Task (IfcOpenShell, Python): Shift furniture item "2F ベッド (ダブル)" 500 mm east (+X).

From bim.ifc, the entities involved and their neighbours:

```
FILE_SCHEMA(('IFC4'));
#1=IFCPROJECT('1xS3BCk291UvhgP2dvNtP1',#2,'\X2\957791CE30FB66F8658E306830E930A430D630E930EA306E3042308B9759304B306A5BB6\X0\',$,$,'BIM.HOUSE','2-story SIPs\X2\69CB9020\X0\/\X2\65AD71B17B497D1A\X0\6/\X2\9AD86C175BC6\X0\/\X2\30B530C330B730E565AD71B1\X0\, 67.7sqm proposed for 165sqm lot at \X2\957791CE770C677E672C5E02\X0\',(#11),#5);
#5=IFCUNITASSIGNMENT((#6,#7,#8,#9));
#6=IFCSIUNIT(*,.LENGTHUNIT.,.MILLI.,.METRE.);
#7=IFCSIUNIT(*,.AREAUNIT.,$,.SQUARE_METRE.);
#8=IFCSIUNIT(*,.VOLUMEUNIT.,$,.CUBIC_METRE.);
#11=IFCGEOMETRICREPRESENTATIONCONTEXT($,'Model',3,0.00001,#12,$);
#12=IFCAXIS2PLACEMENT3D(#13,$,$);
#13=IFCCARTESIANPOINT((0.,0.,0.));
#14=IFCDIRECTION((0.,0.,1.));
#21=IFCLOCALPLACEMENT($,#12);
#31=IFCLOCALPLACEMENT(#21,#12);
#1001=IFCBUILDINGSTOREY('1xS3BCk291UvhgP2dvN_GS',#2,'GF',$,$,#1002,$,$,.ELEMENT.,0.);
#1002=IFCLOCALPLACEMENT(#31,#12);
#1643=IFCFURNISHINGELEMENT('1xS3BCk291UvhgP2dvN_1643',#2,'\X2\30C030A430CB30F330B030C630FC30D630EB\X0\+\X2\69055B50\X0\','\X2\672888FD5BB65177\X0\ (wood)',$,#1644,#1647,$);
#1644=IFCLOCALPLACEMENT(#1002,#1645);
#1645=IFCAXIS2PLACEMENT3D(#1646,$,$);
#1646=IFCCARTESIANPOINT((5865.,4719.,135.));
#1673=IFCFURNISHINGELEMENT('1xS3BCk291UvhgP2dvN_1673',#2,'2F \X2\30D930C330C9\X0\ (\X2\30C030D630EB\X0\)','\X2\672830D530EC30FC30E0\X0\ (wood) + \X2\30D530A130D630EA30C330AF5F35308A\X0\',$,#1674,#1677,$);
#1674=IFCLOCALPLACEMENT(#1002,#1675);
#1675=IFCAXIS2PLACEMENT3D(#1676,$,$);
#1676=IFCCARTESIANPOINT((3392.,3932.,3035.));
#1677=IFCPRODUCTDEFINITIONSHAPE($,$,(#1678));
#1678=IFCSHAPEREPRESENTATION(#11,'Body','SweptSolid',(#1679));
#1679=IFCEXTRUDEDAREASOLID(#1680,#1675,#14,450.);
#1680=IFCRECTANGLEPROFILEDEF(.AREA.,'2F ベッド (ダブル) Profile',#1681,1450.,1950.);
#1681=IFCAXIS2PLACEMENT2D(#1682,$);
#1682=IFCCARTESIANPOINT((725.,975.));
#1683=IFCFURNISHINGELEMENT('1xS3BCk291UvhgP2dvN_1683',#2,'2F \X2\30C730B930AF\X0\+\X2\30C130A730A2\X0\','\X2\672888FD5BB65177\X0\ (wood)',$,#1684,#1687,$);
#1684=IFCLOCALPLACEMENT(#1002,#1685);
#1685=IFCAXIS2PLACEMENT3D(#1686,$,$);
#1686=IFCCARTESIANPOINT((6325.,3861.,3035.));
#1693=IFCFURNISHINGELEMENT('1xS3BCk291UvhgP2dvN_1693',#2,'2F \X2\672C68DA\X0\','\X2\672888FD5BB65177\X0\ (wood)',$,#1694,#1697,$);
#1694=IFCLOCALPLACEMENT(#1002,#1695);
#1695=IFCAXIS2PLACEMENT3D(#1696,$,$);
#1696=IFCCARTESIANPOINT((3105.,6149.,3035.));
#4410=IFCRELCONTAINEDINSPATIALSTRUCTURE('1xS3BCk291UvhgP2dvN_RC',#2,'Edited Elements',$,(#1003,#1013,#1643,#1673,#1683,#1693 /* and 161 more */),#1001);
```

```python
import ifcopenshell
import ifcopenshell.api.geometry
import ifcopenshell.util.placement
import ifcopenshell.util.unit

model = ifcopenshell.open("bim.ifc")
unit_scale = ifcopenshell.util.unit.calculate_unit_scale(model)

item = model.by_id(1673)
matrix = ifcopenshell.util.placement.get_local_placement(item.ObjectPlacement)
matrix[0, 3] += 0.5 / unit_scale
ifcopenshell.api.geometry.edit_object_placement(model, product=item, matrix=matrix, is_si=False)

print(ifcopenshell.util.placement.get_local_placement(item.ObjectPlacement).round(3) + 0.0)

model.write("bim_rev.ifc")
```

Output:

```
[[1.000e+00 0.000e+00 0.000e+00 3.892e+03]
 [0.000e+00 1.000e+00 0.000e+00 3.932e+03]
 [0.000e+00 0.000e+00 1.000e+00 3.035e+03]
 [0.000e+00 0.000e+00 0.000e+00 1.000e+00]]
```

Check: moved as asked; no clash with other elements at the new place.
